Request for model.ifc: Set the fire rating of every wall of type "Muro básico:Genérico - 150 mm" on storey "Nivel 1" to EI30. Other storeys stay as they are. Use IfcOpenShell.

First a look at what the model holds.

```python
import ifcopenshell
import ifcopenshell.util.element

model = ifcopenshell.open("model.ifc")
print(model.schema)
storey = next(s for s in model.by_type("IfcBuildingStorey") if s.Name == "Nivel 1")
walls = [e for e in ifcopenshell.util.element.get_decomposition(storey) if e.is_a("IfcWall")]
seen = {}
for e in walls:
    element_type = ifcopenshell.util.element.get_type(e)
    key = (element_type.Name if element_type != e and element_type else None, ifcopenshell.util.element.get_pset(e, "Pset_WallCommon", "FireRating"))
    seen[key] = seen.get(key, 0) + 1
for (name, value), count in sorted(seen.items(), key=str):
    print(count, "x", name, "|", value)
```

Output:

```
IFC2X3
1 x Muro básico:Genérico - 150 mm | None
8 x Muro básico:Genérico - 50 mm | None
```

```python
import ifcopenshell
import ifcopenshell.api.pset
import ifcopenshell.util.element

model = ifcopenshell.open("model.ifc")

storey = next(s for s in model.by_type("IfcBuildingStorey") if s.Name == "Nivel 1")
walls = [e for e in ifcopenshell.util.element.get_decomposition(storey) if e.is_a("IfcWall")]

count = 0
for e in walls:
    element_type = ifcopenshell.util.element.get_type(e)
    if element_type in (None, e) or element_type.Name != "Muro básico:Genérico - 150 mm":
        continue
    # add_pset returns the element's existing set when there is one.
    pset = ifcopenshell.api.pset.add_pset(model, product=e, name="Pset_WallCommon")
    ifcopenshell.api.pset.edit_pset(model, pset=pset, properties={"FireRating": "EI30"})
    count += 1

print(count, "walls updated")

model.write("model_edited.ifc")
```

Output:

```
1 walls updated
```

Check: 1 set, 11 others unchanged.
